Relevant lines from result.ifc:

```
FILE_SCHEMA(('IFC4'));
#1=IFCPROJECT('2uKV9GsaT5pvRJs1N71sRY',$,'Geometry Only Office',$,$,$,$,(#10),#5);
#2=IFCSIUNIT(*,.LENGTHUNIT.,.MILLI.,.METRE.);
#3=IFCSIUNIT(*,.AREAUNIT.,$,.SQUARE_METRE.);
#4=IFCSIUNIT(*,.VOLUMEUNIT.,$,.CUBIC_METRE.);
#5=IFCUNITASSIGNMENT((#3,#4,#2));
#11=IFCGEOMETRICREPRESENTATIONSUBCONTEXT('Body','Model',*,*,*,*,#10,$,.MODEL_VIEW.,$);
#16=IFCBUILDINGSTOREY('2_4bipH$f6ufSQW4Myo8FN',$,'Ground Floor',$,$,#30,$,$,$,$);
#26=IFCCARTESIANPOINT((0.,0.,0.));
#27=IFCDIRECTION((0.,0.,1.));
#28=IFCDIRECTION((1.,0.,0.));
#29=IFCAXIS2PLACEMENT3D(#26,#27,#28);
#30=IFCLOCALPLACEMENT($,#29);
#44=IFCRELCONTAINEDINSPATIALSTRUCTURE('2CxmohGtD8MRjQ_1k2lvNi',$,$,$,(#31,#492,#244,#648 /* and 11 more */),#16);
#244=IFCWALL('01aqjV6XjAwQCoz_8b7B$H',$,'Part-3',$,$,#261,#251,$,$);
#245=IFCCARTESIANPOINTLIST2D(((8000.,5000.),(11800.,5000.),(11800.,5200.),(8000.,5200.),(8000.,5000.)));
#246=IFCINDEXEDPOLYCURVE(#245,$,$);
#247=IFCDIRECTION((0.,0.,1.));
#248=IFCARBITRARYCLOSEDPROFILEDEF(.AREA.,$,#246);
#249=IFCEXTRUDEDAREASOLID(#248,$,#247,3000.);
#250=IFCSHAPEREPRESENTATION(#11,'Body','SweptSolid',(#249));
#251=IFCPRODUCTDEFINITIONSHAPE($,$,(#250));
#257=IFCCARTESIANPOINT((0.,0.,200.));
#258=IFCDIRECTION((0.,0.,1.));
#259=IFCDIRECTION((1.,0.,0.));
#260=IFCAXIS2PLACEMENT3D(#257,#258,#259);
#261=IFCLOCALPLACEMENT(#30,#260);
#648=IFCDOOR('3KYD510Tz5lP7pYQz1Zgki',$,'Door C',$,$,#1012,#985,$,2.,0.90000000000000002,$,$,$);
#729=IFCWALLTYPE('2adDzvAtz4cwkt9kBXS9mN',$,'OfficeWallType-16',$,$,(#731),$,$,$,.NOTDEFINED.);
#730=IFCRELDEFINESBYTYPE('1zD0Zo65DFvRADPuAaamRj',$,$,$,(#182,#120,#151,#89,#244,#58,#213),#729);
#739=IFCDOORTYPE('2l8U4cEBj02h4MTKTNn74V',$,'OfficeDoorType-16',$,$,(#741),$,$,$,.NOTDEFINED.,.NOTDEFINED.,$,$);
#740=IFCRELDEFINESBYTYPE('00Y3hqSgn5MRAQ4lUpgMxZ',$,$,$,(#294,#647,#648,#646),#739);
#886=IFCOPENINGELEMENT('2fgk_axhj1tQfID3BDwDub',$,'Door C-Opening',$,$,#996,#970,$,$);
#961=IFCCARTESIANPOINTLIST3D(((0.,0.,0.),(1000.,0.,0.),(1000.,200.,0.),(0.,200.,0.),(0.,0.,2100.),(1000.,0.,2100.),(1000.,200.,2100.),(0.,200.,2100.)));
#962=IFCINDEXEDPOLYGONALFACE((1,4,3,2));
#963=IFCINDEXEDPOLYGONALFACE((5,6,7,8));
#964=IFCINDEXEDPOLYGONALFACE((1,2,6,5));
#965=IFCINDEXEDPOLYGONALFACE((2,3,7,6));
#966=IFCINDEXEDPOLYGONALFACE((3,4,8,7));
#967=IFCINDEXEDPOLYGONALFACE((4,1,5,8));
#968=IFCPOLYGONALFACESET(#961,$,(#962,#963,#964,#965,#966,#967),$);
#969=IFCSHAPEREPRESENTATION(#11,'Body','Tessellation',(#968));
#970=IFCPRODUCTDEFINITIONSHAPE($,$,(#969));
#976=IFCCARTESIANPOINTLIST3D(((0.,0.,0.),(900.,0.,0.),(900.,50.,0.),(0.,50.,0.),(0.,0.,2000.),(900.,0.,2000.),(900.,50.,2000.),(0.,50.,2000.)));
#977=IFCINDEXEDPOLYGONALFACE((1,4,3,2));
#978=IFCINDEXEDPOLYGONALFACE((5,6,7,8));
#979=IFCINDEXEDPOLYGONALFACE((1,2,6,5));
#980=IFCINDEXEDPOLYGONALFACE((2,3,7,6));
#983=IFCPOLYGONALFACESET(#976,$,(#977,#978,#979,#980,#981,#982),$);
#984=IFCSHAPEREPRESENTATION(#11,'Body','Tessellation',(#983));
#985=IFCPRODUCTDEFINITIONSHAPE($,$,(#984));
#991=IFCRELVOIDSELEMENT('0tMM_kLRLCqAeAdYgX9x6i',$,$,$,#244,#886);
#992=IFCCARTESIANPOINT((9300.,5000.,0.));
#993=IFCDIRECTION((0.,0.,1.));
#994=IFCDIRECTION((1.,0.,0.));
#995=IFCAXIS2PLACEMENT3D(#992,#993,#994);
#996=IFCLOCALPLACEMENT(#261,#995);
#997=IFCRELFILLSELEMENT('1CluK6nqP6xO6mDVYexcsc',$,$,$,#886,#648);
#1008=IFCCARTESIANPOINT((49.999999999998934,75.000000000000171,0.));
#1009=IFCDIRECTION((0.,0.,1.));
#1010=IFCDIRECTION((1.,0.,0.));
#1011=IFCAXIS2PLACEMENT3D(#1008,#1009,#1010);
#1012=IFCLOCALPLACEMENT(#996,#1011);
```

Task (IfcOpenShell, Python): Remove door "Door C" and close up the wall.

```python
import ifcopenshell
import ifcopenshell.api.feature
import ifcopenshell.api.root
import ifcopenshell.geom
import ifcopenshell.util.shape

model = ifcopenshell.open("result.ifc")
settings = ifcopenshell.geom.settings()


def volume(element):
    """Net volume in cubic metres, openings subtracted."""
    shape = ifcopenshell.geom.create_shape(settings, element)
    return ifcopenshell.util.shape.get_volume(shape.geometry)


door = model.by_guid("3KYD510Tz5lP7pYQz1Zgki")
opening = door.FillsVoids[0].RelatingOpeningElement
wall = opening.VoidsElements[0].RelatingBuildingElement
before = volume(wall)

ifcopenshell.api.root.remove_product(model, product=door)
ifcopenshell.api.feature.remove_feature(model, feature=opening)

after = volume(wall)

print(f"wall volume {before:.3f} -> {after:.3f} m3")

model.write("result_v2.ifc")
```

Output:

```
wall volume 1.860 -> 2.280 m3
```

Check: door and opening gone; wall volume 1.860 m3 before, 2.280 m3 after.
